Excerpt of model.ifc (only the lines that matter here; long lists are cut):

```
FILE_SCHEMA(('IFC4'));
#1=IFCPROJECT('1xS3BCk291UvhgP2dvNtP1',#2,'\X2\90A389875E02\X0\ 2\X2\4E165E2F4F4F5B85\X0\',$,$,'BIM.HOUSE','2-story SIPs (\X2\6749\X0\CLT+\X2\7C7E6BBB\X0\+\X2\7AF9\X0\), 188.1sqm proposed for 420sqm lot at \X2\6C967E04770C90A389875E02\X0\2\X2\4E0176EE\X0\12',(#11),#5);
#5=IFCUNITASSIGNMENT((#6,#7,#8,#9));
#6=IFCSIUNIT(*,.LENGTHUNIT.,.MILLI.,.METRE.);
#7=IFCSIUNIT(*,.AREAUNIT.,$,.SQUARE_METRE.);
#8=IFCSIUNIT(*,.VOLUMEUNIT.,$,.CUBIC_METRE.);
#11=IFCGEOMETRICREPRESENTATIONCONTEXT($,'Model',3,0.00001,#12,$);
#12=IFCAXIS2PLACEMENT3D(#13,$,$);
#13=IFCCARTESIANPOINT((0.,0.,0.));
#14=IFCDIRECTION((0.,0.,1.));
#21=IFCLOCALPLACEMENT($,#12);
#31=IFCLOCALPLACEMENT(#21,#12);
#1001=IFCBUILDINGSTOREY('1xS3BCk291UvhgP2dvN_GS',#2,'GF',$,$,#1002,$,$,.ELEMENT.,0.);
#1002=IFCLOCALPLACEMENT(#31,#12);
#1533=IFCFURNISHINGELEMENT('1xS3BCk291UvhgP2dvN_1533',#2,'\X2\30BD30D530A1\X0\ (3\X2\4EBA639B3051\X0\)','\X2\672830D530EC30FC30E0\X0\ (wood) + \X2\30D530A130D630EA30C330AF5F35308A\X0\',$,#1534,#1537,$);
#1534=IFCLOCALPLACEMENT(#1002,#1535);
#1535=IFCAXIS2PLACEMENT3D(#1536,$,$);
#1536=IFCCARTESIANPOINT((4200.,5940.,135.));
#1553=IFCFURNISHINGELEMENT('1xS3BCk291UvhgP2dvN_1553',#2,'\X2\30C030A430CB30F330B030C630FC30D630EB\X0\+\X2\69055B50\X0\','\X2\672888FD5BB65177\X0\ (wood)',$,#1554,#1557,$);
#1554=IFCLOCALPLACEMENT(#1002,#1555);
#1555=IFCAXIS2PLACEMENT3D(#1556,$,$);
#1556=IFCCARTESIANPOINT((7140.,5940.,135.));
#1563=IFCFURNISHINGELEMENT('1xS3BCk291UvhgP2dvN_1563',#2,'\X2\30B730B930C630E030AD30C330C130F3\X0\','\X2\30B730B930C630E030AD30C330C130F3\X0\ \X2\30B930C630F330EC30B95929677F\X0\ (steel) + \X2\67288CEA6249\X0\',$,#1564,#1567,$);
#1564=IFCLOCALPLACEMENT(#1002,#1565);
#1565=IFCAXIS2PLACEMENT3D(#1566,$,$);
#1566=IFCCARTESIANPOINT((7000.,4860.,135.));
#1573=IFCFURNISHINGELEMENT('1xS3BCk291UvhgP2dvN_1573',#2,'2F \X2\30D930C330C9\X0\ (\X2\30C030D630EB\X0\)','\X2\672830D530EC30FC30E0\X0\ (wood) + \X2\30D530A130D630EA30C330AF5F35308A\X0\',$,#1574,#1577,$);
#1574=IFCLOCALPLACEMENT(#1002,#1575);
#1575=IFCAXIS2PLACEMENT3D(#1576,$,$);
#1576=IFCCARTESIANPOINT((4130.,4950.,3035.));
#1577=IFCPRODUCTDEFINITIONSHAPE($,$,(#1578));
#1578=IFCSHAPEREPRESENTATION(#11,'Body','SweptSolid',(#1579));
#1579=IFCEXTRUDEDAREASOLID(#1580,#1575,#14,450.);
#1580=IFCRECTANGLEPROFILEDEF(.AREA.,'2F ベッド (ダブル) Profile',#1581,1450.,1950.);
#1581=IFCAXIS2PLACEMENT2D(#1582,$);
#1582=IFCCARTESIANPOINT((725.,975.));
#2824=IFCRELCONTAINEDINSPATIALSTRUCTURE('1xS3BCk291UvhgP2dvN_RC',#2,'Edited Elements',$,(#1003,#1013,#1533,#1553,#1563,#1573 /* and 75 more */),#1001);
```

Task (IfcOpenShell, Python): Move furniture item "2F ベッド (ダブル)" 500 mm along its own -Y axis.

```python
import ifcopenshell
import ifcopenshell.api.geometry
import ifcopenshell.util.placement
import ifcopenshell.util.unit

model = ifcopenshell.open("model.ifc")
unit_scale = ifcopenshell.util.unit.calculate_unit_scale(model)

item = model.by_guid("1xS3BCk291UvhgP2dvN_1573")
matrix = ifcopenshell.util.placement.get_local_placement(item.ObjectPlacement)
matrix[:3, 3] -= matrix[:3, 1] * 0.5 / unit_scale
ifcopenshell.api.geometry.edit_object_placement(model, product=item, matrix=matrix, is_si=False)

print(ifcopenshell.util.placement.get_local_placement(item.ObjectPlacement).round(3) + 0.0)

model.write("model_edited.ifc")
```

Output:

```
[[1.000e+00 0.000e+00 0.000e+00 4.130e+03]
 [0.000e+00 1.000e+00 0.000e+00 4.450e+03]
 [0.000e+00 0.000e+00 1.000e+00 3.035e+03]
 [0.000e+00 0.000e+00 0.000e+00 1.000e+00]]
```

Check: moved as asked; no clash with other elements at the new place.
